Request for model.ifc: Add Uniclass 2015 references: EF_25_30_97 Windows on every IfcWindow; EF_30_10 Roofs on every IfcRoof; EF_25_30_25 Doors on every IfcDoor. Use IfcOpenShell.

First a look at what the model holds.

```python
import ifcopenshell

model = ifcopenshell.open("model.ifc")
print(model.schema)
print("classifications:", [c.Name for c in model.by_type("IfcClassification")])
for ifc_class in ("IfcDoor", "IfcRoof", "IfcStair", "IfcWall", "IfcWindow"):
    print(ifc_class, len(model.by_type(ifc_class)))
```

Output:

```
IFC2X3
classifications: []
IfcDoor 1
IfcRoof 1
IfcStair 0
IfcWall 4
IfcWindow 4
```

```python
import ifcopenshell
import ifcopenshell.api.classification

model = ifcopenshell.open("model.ifc")

# IFC2X3 requires Source and Edition and has no link from the project to the system.
system = model.create_entity("IfcClassification", Source="NBS", Edition="2015", Name="Uniclass 2015")

codes = {
    "IfcWindow": ("EF_25_30_97", "Windows"),
    "IfcRoof": ("EF_30_10", "Roofs"),
    "IfcDoor": ("EF_25_30_25", "Doors"),
}
for ifc_class, (code, name) in codes.items():
    products = model.by_type(ifc_class)
    ifcopenshell.api.classification.add_reference(
        model, products=products, classification=system, identification=code, name=name
    )
    print(code, len(products))

model.write("model_edited.ifc")
```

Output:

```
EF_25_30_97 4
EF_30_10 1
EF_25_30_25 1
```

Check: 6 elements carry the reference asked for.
